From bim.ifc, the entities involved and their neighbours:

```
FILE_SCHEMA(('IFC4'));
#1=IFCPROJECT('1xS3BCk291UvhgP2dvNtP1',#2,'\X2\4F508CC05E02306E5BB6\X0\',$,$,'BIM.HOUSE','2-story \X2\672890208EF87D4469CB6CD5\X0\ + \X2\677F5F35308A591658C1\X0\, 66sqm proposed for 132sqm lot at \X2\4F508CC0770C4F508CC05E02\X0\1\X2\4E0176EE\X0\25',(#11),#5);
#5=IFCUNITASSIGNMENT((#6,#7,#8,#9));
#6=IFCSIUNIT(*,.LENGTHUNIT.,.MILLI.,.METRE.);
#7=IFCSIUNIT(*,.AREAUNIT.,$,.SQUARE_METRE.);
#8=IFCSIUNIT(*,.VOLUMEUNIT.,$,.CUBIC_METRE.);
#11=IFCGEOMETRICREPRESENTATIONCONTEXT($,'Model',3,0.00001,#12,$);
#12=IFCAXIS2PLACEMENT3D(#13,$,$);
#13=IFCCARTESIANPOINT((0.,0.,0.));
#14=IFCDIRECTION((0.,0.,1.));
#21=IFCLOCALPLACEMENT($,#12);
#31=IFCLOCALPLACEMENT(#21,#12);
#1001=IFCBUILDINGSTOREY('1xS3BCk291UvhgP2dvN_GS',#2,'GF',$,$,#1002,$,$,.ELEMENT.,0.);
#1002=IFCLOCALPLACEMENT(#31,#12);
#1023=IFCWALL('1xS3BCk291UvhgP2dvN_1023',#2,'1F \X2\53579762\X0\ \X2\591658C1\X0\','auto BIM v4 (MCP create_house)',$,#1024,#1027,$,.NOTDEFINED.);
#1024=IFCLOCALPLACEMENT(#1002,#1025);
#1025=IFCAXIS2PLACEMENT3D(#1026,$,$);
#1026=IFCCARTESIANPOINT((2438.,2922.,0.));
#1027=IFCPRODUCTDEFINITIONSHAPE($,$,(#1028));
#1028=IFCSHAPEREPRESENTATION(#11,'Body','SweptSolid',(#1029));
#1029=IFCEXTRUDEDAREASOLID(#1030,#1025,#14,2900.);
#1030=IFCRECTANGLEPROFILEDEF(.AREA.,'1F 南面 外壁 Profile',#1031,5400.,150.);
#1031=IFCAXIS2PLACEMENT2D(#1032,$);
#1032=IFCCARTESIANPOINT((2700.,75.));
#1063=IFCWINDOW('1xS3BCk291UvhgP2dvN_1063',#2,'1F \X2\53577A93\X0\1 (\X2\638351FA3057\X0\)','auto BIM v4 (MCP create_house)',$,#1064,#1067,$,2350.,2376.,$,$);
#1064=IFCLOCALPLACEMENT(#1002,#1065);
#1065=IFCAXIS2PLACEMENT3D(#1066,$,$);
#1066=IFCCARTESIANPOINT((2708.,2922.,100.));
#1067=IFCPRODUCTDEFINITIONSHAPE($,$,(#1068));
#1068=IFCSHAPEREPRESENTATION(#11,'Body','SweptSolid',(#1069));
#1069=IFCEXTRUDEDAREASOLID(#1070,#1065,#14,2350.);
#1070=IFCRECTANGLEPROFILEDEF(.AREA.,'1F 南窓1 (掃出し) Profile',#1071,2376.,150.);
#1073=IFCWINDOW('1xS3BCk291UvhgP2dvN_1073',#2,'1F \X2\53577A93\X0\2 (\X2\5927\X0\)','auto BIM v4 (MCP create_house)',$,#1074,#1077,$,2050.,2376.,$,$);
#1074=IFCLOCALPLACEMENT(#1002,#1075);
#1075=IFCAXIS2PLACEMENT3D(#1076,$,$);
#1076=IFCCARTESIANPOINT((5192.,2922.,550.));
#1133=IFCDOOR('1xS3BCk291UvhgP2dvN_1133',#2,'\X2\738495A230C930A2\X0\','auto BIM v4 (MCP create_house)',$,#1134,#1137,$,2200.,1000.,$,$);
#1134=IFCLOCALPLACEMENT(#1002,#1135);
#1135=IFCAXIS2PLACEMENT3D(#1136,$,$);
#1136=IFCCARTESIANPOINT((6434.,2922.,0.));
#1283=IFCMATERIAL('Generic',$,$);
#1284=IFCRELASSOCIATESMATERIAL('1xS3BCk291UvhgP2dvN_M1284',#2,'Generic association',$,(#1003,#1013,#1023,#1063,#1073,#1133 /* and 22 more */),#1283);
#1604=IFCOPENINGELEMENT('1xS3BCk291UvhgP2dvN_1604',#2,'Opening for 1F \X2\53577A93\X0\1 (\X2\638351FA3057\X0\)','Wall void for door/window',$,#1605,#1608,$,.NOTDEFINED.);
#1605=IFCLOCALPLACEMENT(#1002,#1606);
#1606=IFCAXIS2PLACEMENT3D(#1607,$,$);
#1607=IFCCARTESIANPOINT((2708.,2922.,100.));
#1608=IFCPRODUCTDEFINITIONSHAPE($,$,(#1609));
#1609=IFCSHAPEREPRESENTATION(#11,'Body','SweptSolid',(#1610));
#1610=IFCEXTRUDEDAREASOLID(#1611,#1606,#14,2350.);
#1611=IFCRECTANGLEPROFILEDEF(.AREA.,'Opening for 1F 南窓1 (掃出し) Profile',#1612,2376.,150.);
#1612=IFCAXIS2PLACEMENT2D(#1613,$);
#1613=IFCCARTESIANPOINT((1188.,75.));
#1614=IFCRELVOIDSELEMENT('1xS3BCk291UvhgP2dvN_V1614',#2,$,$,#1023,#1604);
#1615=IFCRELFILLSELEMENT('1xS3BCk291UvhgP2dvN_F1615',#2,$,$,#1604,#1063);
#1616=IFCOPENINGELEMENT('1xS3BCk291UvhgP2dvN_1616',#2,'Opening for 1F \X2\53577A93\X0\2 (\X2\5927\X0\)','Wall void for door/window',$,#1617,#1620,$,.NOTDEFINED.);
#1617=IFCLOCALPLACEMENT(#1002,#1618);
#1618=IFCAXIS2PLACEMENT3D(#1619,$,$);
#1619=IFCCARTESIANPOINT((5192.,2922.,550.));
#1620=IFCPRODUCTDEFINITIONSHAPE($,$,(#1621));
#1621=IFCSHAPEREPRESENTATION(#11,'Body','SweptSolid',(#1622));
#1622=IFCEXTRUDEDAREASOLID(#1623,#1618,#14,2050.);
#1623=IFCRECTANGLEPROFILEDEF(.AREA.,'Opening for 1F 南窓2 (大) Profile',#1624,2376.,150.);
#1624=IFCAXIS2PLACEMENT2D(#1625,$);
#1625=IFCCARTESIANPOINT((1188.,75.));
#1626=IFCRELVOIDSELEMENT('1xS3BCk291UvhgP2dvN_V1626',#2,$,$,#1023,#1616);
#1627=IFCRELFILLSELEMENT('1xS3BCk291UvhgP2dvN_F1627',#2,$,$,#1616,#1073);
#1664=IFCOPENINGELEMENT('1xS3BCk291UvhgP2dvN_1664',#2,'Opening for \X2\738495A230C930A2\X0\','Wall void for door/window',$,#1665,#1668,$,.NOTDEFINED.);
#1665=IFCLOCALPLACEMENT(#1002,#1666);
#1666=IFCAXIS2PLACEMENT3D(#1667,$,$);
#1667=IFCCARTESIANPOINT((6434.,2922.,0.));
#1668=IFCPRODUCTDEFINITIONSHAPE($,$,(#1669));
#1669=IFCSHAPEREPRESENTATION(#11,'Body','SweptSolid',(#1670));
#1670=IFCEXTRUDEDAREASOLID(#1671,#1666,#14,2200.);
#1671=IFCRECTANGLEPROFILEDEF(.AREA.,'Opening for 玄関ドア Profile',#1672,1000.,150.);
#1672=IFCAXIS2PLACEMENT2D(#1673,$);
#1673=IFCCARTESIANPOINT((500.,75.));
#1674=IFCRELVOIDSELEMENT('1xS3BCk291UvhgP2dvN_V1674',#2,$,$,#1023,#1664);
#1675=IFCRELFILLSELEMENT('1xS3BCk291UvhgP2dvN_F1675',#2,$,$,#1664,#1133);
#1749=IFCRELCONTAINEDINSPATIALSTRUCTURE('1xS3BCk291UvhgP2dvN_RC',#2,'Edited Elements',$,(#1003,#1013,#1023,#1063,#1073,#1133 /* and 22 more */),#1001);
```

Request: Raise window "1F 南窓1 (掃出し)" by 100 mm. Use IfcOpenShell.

```python
import numpy as np
import ifcopenshell
import ifcopenshell.api.geometry
import ifcopenshell.util.placement
import ifcopenshell.util.unit

model = ifcopenshell.open("bim.ifc")
unit_scale = ifcopenshell.util.unit.calculate_unit_scale(model)

window = model.by_id(1063)
opening = window.FillsVoids[0].RelatingOpeningElement
dz = 100.0

shift = np.array([0.0, 0.0, dz])
# The window is not placed relative to its opening, so move both.
for product in (opening, window):
    matrix = ifcopenshell.util.placement.get_local_placement(product.ObjectPlacement)
    matrix[:3, 3] += shift
    ifcopenshell.api.geometry.edit_object_placement(model, product=product, matrix=matrix, is_si=False)

print(f"moved by {dz * unit_scale:+.3f} m")

model.write("bim_updated.ifc")
```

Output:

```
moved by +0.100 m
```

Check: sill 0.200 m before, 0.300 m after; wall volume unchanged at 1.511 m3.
